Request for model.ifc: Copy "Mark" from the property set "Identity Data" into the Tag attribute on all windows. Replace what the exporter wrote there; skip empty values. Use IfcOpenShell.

First a look at what the model holds.

```python
import ifcopenshell
import ifcopenshell.util.element

model = ifcopenshell.open("model.ifc")
print(model.schema)
windows = model.by_type("IfcWindow")
print(len(windows), "windows")
for e in windows[:8]:
    source = ifcopenshell.util.element.get_pset(e, "Identity Data", "Mark")
    target = e.Tag
    print(e.id(), repr(source), repr(target), sep=" | ")
```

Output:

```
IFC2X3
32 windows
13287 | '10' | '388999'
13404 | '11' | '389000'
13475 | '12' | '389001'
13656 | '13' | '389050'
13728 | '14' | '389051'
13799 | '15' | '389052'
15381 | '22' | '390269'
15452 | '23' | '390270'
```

```python
import ifcopenshell
import ifcopenshell.util.element

model = ifcopenshell.open("model.ifc")

count = 0
for e in model.by_type("IfcWindow"):
    value = ifcopenshell.util.element.get_pset(e, "Identity Data", "Mark")
    current = e.Tag
    if not value or not value.strip() or current == value:
        continue
    e.Tag = value
    count += 1

print(count, "windows updated")

model.write("model_updated.ifc")
```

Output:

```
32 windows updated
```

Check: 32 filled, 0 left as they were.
